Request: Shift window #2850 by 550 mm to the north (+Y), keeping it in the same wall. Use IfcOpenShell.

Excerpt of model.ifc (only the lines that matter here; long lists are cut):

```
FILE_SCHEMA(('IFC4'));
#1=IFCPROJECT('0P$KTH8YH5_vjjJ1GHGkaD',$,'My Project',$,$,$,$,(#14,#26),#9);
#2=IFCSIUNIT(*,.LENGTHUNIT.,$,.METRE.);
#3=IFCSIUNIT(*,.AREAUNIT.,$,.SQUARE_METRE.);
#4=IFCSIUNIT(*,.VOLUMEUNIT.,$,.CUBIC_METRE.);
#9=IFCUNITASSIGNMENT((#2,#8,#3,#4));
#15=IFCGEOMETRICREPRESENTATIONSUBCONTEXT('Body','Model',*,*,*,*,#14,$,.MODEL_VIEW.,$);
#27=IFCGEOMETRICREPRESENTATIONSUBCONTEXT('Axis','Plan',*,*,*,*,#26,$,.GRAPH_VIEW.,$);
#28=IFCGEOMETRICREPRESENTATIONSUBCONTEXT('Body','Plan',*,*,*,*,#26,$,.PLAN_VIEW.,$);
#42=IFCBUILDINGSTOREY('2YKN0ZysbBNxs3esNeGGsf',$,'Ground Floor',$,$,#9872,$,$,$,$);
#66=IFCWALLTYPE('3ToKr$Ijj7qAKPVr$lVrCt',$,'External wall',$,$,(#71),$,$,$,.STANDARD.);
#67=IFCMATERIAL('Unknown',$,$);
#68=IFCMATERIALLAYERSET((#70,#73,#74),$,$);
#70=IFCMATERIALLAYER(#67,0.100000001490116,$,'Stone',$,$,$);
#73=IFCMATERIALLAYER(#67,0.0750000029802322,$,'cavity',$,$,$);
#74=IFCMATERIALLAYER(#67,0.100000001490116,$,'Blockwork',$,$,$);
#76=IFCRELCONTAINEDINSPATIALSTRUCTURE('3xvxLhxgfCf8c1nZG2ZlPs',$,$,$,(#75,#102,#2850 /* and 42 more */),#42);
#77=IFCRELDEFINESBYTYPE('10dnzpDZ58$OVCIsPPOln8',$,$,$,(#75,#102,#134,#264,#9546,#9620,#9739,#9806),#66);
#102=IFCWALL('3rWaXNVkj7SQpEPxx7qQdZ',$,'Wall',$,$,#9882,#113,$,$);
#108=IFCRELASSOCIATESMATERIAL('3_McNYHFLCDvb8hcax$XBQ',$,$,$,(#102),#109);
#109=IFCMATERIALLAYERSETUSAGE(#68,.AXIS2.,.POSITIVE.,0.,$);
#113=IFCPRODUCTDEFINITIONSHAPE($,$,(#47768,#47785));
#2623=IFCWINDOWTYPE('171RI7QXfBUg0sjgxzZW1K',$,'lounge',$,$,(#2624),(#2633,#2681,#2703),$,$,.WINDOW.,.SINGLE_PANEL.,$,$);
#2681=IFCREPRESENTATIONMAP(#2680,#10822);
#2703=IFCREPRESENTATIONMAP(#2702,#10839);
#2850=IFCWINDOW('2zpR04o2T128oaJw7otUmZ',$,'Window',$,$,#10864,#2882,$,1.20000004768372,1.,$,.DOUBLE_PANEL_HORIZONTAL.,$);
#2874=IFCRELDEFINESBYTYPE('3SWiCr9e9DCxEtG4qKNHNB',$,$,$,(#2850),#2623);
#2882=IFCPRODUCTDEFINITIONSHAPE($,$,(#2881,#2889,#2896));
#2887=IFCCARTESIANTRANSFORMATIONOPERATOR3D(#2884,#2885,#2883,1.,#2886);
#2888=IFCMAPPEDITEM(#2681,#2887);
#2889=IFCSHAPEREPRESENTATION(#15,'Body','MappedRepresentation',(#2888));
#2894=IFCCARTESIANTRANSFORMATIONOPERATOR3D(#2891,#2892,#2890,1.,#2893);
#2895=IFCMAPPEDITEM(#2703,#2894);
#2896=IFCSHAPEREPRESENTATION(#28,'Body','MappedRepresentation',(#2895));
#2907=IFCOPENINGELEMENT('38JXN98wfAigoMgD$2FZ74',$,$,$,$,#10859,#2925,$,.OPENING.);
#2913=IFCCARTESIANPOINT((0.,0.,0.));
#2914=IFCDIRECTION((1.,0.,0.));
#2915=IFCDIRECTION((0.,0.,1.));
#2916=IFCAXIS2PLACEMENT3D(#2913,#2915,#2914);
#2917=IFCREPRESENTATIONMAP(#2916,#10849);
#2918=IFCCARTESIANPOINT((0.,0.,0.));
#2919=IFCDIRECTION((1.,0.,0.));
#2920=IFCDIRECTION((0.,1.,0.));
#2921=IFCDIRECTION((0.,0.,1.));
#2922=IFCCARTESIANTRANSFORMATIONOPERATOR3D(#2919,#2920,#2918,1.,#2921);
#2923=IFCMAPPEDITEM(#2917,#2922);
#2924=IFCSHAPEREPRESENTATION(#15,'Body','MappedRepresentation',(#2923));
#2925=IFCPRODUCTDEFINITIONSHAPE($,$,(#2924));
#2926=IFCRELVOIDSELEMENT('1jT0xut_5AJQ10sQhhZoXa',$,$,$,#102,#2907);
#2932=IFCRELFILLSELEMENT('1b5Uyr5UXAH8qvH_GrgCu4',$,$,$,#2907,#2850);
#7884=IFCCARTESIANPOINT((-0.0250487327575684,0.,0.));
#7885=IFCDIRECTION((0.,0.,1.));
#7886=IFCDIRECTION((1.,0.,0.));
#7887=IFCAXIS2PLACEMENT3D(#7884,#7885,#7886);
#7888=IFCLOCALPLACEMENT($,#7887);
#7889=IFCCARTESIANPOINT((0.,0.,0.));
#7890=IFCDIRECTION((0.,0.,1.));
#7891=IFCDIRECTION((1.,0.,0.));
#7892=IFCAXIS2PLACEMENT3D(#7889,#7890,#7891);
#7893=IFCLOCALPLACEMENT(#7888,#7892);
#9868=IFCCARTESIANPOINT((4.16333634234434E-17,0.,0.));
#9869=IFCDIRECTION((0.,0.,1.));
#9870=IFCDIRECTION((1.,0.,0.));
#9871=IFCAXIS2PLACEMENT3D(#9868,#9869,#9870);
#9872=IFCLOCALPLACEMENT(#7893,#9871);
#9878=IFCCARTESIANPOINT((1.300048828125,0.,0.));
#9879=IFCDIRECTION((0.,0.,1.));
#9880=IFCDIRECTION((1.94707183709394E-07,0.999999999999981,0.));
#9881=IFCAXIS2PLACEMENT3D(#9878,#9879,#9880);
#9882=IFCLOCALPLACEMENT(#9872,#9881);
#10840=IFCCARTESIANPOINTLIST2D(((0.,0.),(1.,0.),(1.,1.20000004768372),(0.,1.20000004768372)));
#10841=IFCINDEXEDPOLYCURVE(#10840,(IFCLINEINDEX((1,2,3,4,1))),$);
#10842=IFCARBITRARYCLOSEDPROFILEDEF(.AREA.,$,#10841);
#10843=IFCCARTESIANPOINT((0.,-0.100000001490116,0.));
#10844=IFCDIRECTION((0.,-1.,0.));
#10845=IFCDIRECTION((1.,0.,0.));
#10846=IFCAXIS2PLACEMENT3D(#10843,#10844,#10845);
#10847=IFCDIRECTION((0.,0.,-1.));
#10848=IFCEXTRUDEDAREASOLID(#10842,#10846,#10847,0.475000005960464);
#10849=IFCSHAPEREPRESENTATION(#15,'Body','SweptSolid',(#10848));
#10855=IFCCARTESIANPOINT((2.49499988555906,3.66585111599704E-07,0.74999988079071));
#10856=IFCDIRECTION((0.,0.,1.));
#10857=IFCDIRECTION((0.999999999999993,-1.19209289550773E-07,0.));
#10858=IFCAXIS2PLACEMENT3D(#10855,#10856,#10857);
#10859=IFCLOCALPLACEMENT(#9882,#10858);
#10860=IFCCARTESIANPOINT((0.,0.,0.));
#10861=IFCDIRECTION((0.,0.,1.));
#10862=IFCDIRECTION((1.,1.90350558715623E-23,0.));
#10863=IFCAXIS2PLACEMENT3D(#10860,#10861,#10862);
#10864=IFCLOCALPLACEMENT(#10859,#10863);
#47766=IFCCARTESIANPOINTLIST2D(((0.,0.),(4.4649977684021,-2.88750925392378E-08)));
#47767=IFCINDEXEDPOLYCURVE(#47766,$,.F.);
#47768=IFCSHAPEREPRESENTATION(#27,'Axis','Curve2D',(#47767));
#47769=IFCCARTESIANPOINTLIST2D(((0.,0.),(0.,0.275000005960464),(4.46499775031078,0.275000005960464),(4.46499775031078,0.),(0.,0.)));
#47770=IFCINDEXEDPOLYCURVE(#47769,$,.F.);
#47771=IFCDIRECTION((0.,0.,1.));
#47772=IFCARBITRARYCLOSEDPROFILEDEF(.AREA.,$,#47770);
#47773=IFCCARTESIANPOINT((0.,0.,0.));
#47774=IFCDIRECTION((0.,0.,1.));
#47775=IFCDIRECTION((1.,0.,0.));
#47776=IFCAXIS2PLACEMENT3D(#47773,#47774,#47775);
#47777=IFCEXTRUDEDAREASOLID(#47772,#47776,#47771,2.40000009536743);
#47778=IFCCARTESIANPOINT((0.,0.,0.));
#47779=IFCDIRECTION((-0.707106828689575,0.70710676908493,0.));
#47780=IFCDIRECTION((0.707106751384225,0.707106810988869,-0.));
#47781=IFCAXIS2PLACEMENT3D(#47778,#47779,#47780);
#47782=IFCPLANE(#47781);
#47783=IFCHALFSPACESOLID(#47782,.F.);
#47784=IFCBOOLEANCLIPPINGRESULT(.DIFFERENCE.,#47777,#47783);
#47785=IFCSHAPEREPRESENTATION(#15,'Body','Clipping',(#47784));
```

```python
import ifcopenshell
import ifcopenshell.api.geometry
import ifcopenshell.util.placement

model = ifcopenshell.open("model.ifc")

window = model.by_id(2850)
opening = window.FillsVoids[0].RelatingOpeningElement
wall = opening.VoidsElements[0].RelatingBuildingElement

wall_matrix = ifcopenshell.util.placement.get_local_placement(wall.ObjectPlacement)
shift = wall_matrix[:3, 0] * 0.55
before = ifcopenshell.util.placement.get_local_placement(window.ObjectPlacement)[:3, 3].copy()

# The window is placed relative to its opening, so it follows when the opening moves.
matrix = ifcopenshell.util.placement.get_local_placement(opening.ObjectPlacement)
matrix[:3, 3] += shift
ifcopenshell.api.geometry.edit_object_placement(
    model, product=opening, matrix=matrix, is_si=False, should_transform_children=True
)

after = ifcopenshell.util.placement.get_local_placement(window.ObjectPlacement)[:3, 3]
print("window moved by", (after - before).round(3) + 0.0)

model.write("model-out.ifc")
```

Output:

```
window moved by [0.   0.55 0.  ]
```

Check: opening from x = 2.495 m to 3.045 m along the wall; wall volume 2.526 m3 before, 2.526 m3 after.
